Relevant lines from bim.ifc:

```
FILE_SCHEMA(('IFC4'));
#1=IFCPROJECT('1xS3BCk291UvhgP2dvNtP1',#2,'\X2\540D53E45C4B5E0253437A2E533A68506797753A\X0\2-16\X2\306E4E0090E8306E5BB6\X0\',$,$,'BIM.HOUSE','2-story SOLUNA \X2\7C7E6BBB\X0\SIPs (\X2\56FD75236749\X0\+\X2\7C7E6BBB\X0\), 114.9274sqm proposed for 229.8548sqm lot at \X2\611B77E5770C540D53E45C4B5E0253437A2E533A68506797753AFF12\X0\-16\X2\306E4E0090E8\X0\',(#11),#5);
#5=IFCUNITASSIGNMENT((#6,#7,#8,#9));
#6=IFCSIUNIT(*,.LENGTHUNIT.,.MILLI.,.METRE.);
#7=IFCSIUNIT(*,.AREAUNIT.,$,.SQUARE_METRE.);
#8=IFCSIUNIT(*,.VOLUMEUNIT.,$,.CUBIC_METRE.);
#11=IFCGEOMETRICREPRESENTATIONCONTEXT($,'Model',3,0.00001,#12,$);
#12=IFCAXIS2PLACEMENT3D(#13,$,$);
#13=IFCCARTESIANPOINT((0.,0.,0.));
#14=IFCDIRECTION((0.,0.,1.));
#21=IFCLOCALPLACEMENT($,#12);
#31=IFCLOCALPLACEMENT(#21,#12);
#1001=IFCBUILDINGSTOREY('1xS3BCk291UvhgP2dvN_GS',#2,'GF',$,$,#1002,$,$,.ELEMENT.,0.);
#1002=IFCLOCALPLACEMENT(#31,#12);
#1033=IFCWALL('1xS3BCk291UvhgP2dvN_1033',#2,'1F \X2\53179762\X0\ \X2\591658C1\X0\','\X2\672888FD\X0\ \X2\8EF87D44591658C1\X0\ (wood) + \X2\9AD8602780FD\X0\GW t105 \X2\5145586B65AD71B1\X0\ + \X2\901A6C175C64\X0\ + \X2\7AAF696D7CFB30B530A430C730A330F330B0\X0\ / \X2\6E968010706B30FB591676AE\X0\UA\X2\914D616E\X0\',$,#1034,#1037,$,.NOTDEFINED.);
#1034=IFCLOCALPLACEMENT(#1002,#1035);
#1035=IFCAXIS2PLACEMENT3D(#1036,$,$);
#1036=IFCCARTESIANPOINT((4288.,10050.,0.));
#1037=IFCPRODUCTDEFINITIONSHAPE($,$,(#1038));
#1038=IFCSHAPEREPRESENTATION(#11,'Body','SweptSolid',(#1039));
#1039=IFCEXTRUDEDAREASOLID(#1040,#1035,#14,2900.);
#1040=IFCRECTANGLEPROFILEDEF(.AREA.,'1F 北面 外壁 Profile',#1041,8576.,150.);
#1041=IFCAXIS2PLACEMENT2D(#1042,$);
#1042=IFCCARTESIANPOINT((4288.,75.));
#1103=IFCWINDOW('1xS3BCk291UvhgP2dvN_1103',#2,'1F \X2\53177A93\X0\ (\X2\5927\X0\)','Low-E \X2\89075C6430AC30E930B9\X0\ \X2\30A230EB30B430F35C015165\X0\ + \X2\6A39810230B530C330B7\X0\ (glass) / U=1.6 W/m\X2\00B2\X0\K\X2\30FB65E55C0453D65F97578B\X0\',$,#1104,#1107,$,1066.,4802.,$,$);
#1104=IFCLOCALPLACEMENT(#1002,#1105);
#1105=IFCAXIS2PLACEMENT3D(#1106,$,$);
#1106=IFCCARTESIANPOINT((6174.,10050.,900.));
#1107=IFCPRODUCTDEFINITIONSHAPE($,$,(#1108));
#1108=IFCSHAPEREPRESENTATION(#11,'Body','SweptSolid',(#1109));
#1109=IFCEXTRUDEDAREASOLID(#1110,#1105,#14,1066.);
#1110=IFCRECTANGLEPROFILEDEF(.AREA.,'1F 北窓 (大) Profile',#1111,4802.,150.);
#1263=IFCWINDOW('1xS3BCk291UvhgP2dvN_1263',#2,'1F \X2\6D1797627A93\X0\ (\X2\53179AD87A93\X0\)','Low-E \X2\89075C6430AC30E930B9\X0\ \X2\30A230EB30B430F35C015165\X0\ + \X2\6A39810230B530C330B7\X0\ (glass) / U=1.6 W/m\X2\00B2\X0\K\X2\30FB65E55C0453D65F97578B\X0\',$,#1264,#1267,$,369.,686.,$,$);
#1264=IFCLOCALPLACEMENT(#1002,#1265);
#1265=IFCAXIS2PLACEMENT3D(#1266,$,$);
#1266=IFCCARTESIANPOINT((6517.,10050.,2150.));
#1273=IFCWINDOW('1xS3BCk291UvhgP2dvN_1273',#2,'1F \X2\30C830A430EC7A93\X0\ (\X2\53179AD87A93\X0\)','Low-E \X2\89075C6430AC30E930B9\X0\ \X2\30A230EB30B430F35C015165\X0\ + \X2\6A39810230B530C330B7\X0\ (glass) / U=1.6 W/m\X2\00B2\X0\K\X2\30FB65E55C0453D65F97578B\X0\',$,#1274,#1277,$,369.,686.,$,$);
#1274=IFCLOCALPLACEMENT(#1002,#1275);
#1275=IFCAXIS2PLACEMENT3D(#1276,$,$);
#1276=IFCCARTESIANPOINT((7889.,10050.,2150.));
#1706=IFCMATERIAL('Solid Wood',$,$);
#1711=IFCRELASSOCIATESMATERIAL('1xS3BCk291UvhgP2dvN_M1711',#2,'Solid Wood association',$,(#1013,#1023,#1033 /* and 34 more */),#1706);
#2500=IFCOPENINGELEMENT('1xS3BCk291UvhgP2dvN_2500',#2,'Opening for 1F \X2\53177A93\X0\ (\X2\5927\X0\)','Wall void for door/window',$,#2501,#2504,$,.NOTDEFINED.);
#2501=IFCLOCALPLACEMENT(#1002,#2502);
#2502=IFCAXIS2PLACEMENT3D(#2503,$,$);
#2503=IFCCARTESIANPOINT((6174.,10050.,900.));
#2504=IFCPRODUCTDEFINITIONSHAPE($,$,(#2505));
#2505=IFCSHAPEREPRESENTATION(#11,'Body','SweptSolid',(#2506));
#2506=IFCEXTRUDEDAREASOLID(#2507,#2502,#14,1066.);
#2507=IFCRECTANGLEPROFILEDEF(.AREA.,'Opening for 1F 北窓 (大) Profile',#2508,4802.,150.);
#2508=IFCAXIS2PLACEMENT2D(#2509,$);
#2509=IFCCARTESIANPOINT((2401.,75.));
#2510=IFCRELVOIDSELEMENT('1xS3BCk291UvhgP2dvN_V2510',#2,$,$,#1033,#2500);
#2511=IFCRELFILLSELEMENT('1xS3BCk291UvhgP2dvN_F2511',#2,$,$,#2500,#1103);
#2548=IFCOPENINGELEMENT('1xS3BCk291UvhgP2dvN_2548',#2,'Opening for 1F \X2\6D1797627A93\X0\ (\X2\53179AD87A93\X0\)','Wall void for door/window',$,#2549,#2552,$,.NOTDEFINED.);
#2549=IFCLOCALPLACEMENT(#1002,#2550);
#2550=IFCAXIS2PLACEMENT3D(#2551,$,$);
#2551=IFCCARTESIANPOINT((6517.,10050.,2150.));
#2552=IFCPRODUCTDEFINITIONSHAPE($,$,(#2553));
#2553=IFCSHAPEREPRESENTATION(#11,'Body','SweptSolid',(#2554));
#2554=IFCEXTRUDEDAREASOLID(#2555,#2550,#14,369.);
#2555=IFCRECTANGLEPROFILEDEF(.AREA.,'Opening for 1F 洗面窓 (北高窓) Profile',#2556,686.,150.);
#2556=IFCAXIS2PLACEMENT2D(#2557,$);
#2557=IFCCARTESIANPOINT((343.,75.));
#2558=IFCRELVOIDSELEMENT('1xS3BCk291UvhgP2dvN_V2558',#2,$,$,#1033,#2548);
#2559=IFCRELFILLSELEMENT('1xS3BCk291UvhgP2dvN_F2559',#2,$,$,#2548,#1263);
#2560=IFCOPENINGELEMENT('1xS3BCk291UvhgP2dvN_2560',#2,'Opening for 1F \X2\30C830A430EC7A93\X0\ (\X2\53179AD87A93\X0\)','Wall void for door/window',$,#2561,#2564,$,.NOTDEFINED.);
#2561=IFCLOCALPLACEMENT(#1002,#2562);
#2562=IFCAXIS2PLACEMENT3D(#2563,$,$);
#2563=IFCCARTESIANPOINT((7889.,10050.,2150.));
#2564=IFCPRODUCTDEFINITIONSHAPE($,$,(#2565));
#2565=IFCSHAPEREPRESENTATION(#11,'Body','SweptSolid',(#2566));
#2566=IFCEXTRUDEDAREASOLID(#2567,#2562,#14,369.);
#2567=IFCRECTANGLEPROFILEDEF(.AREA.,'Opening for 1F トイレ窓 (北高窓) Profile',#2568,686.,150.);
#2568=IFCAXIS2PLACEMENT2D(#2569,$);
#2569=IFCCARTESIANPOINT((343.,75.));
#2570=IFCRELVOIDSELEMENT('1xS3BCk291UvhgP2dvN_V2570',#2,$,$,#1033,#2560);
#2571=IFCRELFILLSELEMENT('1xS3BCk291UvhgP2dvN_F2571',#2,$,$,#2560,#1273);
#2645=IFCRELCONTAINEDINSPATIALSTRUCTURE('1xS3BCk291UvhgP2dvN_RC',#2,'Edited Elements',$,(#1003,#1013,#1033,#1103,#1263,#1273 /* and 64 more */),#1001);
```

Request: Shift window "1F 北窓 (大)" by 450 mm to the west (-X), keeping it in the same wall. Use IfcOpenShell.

```python
import ifcopenshell
import ifcopenshell.api.geometry
import ifcopenshell.util.placement
import ifcopenshell.util.unit

model = ifcopenshell.open("bim.ifc")
unit_scale = ifcopenshell.util.unit.calculate_unit_scale(model)

window = model.by_guid("1xS3BCk291UvhgP2dvN_1103")
opening = window.FillsVoids[0].RelatingOpeningElement
wall = opening.VoidsElements[0].RelatingBuildingElement

wall_matrix = ifcopenshell.util.placement.get_local_placement(wall.ObjectPlacement)
shift = wall_matrix[:3, 0] * -0.45 / unit_scale
before = ifcopenshell.util.placement.get_local_placement(window.ObjectPlacement)[:3, 3].copy()

# The window is not placed relative to its opening, so move both.
for product in (opening, window):
    matrix = ifcopenshell.util.placement.get_local_placement(product.ObjectPlacement)
    matrix[:3, 3] += shift
    ifcopenshell.api.geometry.edit_object_placement(model, product=product, matrix=matrix, is_si=False)

after = ifcopenshell.util.placement.get_local_placement(window.ObjectPlacement)[:3, 3]
print("window moved by", (after - before).round(3) + 0.0)

model.write("bim_edited.ifc")
```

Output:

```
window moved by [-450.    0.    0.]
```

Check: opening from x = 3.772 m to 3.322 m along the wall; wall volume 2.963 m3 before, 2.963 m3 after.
